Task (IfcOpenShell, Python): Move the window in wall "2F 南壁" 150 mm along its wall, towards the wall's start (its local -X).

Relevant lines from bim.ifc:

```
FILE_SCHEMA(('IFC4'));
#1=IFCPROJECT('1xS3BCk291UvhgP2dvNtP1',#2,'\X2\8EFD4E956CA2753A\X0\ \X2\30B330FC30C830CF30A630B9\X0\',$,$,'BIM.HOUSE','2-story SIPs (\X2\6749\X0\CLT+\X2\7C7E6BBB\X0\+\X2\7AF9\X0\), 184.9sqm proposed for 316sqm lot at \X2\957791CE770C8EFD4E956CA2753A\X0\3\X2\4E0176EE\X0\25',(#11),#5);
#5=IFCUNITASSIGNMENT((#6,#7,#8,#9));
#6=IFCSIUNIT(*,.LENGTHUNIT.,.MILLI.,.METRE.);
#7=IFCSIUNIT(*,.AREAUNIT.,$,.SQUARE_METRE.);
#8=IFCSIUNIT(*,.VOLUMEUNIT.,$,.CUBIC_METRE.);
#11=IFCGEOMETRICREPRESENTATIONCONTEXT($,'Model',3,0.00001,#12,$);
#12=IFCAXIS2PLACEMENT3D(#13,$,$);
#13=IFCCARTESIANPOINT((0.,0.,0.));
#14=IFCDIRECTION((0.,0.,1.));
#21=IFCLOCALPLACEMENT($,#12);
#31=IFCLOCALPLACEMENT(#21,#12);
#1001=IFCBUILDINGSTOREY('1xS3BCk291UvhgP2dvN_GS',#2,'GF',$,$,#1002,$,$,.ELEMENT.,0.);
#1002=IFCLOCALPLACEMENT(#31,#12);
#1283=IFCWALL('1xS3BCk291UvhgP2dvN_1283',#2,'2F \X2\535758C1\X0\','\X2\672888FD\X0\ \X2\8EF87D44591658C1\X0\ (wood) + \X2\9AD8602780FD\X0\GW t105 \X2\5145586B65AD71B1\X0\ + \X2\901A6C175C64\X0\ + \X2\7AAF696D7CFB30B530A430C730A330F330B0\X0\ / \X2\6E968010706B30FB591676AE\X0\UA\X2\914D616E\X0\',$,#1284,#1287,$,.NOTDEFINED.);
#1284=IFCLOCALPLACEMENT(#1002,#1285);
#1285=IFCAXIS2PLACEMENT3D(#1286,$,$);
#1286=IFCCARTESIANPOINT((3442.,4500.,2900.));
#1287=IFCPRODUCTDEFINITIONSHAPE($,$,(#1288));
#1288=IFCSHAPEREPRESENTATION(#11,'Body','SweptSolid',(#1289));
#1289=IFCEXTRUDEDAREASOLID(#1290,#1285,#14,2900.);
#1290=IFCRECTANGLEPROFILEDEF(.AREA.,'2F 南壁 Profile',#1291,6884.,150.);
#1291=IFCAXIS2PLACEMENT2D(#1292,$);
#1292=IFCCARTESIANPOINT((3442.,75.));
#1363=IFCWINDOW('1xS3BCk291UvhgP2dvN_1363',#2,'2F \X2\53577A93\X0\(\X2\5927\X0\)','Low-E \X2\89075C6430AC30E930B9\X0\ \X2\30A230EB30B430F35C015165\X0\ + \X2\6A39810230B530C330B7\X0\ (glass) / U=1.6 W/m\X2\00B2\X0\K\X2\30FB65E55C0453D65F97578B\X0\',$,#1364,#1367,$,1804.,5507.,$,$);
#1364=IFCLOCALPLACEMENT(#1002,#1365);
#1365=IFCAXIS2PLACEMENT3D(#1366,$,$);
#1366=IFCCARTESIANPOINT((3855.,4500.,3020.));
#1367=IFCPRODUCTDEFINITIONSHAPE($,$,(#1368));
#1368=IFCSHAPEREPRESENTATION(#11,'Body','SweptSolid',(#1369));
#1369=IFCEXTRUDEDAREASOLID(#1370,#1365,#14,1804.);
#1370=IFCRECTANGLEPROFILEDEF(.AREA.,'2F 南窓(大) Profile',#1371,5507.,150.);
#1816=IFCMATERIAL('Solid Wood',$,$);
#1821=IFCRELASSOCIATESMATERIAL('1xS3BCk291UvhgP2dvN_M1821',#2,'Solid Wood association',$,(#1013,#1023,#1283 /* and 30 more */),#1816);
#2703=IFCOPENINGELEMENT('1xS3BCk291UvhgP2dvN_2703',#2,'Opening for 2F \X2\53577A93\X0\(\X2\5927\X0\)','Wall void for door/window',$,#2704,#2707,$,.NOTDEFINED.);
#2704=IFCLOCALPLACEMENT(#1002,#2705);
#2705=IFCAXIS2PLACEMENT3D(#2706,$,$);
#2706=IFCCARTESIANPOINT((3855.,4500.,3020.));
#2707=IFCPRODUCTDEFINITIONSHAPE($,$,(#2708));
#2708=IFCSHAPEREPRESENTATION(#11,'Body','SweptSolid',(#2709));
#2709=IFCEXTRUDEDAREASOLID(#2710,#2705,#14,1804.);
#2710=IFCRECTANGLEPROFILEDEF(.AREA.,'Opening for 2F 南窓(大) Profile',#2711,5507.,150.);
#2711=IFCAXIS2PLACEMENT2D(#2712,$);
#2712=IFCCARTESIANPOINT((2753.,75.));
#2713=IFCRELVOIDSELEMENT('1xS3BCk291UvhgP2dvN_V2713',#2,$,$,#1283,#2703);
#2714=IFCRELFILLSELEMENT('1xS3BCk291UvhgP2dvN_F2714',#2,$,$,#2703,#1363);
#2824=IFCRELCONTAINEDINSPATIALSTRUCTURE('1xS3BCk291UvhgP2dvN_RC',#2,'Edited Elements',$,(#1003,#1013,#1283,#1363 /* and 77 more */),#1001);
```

```python
import ifcopenshell
import ifcopenshell.api.geometry
import ifcopenshell.util.placement
import ifcopenshell.util.unit

model = ifcopenshell.open("bim.ifc")
unit_scale = ifcopenshell.util.unit.calculate_unit_scale(model)

window = model.by_guid("1xS3BCk291UvhgP2dvN_1363")
opening = window.FillsVoids[0].RelatingOpeningElement
wall = opening.VoidsElements[0].RelatingBuildingElement

wall_matrix = ifcopenshell.util.placement.get_local_placement(wall.ObjectPlacement)
shift = wall_matrix[:3, 0] * -0.15 / unit_scale
before = ifcopenshell.util.placement.get_local_placement(window.ObjectPlacement)[:3, 3].copy()

# The window is not placed relative to its opening, so move both.
for product in (opening, window):
    matrix = ifcopenshell.util.placement.get_local_placement(product.ObjectPlacement)
    matrix[:3, 3] += shift
    ifcopenshell.api.geometry.edit_object_placement(model, product=product, matrix=matrix, is_si=False)

after = ifcopenshell.util.placement.get_local_placement(window.ObjectPlacement)[:3, 3]
print("window moved by", (after - before).round(3) + 0.0)

model.write("bim-out.ifc")
```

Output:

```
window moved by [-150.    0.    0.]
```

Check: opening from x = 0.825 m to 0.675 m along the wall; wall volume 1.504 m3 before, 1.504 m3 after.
